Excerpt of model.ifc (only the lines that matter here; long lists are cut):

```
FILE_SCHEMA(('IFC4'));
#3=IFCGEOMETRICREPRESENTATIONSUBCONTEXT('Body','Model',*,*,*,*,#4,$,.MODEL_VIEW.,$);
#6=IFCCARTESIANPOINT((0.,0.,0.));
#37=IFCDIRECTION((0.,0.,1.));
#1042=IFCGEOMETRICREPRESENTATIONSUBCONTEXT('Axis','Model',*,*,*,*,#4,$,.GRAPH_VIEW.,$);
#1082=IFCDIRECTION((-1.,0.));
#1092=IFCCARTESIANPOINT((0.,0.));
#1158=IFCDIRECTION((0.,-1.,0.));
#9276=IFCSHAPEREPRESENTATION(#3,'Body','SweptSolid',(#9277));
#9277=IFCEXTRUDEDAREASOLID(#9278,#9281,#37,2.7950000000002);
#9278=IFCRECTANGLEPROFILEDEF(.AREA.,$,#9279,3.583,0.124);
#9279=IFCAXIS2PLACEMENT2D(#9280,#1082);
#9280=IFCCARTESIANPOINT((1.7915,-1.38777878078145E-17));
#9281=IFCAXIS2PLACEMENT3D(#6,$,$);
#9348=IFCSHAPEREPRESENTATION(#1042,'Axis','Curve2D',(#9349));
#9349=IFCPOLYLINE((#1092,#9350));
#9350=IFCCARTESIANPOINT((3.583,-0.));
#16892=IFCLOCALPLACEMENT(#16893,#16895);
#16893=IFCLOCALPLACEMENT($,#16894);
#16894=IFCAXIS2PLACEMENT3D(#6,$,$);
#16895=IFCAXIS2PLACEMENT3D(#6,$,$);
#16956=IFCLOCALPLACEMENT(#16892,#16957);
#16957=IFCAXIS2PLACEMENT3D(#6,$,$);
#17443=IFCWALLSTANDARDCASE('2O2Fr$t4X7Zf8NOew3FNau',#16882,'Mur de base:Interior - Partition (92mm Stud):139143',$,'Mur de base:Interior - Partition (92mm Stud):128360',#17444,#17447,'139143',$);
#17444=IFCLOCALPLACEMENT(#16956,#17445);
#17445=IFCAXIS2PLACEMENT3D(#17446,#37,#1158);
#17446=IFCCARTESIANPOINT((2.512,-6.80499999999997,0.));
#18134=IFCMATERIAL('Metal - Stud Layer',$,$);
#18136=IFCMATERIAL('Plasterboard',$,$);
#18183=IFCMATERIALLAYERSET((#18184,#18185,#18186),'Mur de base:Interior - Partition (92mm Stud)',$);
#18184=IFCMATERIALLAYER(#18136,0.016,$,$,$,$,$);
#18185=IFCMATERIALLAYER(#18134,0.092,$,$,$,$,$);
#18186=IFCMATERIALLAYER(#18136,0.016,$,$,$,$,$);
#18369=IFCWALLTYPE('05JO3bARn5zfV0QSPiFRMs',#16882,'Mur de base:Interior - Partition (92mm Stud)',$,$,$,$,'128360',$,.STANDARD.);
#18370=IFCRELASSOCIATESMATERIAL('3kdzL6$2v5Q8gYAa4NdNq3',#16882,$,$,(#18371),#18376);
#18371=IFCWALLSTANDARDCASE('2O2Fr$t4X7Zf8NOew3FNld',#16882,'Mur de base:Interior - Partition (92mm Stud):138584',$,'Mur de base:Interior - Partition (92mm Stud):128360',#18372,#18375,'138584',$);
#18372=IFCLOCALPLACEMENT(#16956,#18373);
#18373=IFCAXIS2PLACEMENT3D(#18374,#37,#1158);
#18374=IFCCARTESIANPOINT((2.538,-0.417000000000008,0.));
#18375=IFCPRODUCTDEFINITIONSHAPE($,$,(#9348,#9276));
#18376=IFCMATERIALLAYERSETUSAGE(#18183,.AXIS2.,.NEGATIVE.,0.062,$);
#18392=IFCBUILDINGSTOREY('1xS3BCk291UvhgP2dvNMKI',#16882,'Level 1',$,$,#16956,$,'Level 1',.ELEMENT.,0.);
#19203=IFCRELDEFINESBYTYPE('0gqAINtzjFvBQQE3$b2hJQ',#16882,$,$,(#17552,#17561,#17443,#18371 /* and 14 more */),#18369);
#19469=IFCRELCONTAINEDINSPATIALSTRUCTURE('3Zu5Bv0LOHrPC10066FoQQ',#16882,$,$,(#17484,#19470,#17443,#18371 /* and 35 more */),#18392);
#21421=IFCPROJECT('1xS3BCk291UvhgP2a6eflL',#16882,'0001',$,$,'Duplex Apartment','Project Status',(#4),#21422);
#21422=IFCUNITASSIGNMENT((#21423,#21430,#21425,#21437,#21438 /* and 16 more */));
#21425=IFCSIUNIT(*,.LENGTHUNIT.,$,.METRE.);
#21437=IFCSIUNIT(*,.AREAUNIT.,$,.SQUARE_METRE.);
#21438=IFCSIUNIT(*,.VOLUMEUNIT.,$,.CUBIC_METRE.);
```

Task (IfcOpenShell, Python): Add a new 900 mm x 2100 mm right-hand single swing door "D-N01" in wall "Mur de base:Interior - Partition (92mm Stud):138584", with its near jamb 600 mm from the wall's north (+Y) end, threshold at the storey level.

```python
import numpy as np
import ifcopenshell
import ifcopenshell.api.feature
import ifcopenshell.api.geometry
import ifcopenshell.api.root
import ifcopenshell.api.spatial
import ifcopenshell.geom
import ifcopenshell.util.element
import ifcopenshell.util.placement
import ifcopenshell.util.representation
import ifcopenshell.util.shape
import ifcopenshell.util.unit

model = ifcopenshell.open("model.ifc")
unit_scale = ifcopenshell.util.unit.calculate_unit_scale(model)
settings = ifcopenshell.geom.settings()


def volume(element):
    """Net volume in cubic metres, openings subtracted."""
    shape = ifcopenshell.geom.create_shape(settings, element)
    return ifcopenshell.util.shape.get_volume(shape.geometry)


wall = model.by_id(18371)
storey = ifcopenshell.util.element.get_container(wall, ifc_class="IfcBuildingStorey")
context = ifcopenshell.util.representation.get_context(model, "Model", "Body", "MODEL_VIEW")
before = volume(wall)

width, height, from_end, sill = 0.9, 2.1, 0.6, 0.0  # metres

# The wall runs along its own X axis, and the end named is its -X end.
wall_shape = ifcopenshell.geom.create_shape(settings, wall)
x, y, z = ifcopenshell.util.shape.get_vertices(wall_shape.geometry).T
start = x.min() + from_end
face, thickness = float(y.min()), float(y.max() - y.min())
wall_matrix = ifcopenshell.util.placement.get_local_placement(wall.ObjectPlacement)
level = ifcopenshell.util.placement.get_local_placement(storey.ObjectPlacement)[2, 3]


def in_wall(x, y):
    """Placement at x, y metres in the wall's axes, at sill height."""
    matrix = wall_matrix.copy()
    matrix[:, 3] = wall_matrix @ np.array([x / unit_scale, y / unit_scale, 0.0, 1.0])
    matrix[2, 3] = level + sill / unit_scale
    return matrix


# Opening: a box that overshoots both wall faces by 50 mm.
opening = ifcopenshell.api.root.create_entity(model, ifc_class="IfcOpeningElement", predefined_type="OPENING")
box = ifcopenshell.api.geometry.add_wall_representation(
    model, context=context, length=width, height=height, thickness=thickness + 0.1
)
ifcopenshell.api.geometry.assign_representation(model, product=opening, representation=box)
ifcopenshell.api.geometry.edit_object_placement(model, product=opening, matrix=in_wall(start, face - 0.05), is_si=False)
ifcopenshell.api.feature.add_feature(model, feature=opening, element=wall)

door = ifcopenshell.api.root.create_entity(model, ifc_class="IfcDoor", name="D-N01", predefined_type="DOOR")
door.OverallWidth, door.OverallHeight = width / unit_scale, height / unit_scale
door.OperationType = "SINGLE_SWING_RIGHT"
body = ifcopenshell.api.geometry.add_door_representation(
    model,
    context=context,
    overall_width=door.OverallWidth,
    overall_height=door.OverallHeight,
    operation_type="SINGLE_SWING_RIGHT",
    lining_properties={"LiningDepth": thickness / unit_scale, "ThresholdDepth": thickness / unit_scale},
)
ifcopenshell.api.geometry.assign_representation(model, product=door, representation=body)
ifcopenshell.api.spatial.assign_container(model, products=[door], relating_structure=storey)
ifcopenshell.api.feature.add_filling(model, opening=opening, element=door)

# The lining spans the wall, so the door starts at the wall face.
ifcopenshell.api.geometry.edit_object_placement(model, product=door, matrix=in_wall(start, face), is_si=False)

after = volume(wall)

print(f"wall volume {before:.3f} -> {after:.3f} m3")

model.write("model-out.ifc")
```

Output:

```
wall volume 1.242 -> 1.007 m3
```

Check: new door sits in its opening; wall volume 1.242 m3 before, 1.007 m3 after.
